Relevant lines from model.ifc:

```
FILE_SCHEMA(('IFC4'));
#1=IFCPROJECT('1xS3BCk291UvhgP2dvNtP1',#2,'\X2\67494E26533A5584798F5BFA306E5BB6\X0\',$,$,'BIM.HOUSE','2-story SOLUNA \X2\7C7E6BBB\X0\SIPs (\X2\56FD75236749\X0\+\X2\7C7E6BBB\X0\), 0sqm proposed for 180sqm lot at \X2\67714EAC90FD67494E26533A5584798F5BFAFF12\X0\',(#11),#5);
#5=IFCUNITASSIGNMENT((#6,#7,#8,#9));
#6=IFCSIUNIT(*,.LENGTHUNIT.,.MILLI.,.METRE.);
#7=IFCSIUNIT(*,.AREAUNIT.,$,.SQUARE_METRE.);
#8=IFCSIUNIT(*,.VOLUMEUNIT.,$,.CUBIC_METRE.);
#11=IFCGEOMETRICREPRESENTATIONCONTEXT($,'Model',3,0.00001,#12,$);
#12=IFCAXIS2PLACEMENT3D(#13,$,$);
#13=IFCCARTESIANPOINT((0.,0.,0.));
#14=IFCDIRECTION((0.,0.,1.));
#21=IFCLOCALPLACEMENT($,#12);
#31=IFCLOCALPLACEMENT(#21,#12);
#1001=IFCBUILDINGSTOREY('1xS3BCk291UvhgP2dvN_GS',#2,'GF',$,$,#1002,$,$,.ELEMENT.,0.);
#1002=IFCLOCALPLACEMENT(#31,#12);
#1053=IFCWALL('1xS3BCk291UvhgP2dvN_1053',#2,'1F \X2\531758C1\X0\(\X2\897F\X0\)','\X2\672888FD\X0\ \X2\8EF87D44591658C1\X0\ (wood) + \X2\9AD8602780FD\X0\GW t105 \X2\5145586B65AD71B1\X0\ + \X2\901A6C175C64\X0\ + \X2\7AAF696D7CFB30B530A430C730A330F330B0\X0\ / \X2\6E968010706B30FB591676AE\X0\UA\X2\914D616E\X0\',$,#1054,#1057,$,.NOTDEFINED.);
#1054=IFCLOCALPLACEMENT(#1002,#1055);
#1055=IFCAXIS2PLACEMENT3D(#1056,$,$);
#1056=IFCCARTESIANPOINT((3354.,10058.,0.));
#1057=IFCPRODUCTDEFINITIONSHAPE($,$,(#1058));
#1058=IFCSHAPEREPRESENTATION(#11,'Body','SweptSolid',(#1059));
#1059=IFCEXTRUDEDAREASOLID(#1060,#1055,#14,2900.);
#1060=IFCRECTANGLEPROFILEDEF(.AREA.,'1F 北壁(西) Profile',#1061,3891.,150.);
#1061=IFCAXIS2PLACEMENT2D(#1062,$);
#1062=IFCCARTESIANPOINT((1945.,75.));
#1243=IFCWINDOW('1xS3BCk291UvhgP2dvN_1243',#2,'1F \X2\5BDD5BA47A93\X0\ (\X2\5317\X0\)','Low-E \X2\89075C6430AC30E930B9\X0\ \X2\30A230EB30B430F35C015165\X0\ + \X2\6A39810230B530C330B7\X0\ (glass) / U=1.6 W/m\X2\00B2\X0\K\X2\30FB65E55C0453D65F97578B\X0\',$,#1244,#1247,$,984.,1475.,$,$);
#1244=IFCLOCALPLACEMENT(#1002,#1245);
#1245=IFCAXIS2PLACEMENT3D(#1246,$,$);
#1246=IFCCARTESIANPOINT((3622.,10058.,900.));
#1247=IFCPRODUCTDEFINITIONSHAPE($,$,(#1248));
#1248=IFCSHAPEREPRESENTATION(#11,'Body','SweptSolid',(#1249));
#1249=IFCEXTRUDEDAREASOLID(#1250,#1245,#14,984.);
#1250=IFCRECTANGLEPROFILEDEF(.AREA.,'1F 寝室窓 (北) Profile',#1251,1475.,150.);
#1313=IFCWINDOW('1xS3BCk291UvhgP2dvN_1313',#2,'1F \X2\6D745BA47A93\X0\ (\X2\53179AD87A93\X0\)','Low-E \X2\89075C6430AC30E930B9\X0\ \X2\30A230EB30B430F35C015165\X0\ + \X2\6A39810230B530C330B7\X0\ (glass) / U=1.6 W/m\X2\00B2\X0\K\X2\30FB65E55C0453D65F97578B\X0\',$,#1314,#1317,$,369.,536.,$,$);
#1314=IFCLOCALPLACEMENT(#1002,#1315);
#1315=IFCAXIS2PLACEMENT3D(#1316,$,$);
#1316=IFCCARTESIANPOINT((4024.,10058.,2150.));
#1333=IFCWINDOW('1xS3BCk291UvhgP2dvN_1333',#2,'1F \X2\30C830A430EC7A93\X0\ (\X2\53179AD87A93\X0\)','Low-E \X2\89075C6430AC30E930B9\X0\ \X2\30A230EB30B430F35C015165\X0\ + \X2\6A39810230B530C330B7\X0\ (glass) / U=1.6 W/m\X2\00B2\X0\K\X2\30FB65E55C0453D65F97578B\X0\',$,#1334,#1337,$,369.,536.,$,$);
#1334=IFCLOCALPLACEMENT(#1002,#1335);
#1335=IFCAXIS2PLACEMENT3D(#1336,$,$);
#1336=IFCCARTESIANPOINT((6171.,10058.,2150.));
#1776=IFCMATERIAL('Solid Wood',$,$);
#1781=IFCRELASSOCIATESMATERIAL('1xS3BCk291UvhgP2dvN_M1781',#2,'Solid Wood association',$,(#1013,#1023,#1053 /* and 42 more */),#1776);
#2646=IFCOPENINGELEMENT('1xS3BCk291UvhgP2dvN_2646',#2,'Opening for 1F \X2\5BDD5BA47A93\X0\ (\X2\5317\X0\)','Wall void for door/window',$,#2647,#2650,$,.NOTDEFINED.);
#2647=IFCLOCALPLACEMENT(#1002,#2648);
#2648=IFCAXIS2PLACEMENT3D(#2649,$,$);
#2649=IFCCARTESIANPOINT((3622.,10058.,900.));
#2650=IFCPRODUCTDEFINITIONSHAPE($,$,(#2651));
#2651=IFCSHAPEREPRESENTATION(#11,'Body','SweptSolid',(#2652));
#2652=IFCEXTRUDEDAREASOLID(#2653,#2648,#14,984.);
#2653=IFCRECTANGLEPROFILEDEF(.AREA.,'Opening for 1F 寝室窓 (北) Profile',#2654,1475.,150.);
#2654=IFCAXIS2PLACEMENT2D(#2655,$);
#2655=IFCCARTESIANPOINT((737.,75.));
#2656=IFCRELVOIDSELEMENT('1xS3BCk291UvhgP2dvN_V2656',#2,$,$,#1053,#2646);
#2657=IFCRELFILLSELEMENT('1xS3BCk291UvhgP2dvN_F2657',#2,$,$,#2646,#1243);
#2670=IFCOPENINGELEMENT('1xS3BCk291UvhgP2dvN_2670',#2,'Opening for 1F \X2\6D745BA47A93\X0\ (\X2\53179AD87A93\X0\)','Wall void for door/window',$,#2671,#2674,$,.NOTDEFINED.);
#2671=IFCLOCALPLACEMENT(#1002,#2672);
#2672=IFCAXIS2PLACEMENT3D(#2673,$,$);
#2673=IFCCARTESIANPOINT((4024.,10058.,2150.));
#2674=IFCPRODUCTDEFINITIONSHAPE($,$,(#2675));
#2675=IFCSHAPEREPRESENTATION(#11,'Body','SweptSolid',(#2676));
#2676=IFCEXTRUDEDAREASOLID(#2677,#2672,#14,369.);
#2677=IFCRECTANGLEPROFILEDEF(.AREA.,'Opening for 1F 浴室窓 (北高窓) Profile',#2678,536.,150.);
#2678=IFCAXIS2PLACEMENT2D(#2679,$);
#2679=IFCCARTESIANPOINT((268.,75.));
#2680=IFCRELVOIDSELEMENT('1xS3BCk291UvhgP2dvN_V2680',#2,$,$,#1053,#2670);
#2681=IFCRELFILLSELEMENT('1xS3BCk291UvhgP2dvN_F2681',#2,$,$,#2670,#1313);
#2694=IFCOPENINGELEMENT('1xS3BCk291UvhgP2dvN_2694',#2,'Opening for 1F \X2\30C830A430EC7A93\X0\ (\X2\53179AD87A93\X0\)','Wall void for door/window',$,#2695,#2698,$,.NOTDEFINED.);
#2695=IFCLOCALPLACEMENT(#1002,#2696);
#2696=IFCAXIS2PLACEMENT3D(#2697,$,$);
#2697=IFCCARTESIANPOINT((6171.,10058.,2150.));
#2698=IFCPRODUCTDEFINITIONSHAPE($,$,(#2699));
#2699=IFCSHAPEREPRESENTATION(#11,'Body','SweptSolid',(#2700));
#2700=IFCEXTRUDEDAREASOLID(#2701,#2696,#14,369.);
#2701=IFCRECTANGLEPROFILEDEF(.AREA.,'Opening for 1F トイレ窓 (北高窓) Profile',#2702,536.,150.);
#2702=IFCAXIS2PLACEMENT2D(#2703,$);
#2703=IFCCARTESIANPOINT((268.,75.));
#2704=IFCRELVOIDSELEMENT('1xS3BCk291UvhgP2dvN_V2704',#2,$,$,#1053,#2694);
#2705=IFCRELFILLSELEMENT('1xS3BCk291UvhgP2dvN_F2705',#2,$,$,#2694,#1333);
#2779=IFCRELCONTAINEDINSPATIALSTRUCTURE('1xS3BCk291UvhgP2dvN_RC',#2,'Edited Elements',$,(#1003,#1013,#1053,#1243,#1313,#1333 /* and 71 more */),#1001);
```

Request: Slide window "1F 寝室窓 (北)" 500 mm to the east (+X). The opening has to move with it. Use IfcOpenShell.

```python
import ifcopenshell
import ifcopenshell.api.geometry
import ifcopenshell.util.placement

model = ifcopenshell.open("model.ifc")

window = model.by_guid("1xS3BCk291UvhgP2dvN_1243")
opening = window.FillsVoids[0].RelatingOpeningElement
wall = opening.VoidsElements[0].RelatingBuildingElement

wall_matrix = ifcopenshell.util.placement.get_local_placement(wall.ObjectPlacement)
shift = wall_matrix[:3, 0] * 500.0
before = ifcopenshell.util.placement.get_local_placement(window.ObjectPlacement)[:3, 3].copy()

# The window is not placed relative to its opening, so move both.
for product in (opening, window):
    matrix = ifcopenshell.util.placement.get_local_placement(product.ObjectPlacement)
    matrix[:3, 3] += shift
    ifcopenshell.api.geometry.edit_object_placement(model, product=product, matrix=matrix, is_si=False)

after = ifcopenshell.util.placement.get_local_placement(window.ObjectPlacement)[:3, 3]
print("window moved by", (after - before).round(3) + 0.0)

model.write("model_v2.ifc")
```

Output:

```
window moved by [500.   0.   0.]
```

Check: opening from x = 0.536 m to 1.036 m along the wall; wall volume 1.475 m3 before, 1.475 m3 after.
